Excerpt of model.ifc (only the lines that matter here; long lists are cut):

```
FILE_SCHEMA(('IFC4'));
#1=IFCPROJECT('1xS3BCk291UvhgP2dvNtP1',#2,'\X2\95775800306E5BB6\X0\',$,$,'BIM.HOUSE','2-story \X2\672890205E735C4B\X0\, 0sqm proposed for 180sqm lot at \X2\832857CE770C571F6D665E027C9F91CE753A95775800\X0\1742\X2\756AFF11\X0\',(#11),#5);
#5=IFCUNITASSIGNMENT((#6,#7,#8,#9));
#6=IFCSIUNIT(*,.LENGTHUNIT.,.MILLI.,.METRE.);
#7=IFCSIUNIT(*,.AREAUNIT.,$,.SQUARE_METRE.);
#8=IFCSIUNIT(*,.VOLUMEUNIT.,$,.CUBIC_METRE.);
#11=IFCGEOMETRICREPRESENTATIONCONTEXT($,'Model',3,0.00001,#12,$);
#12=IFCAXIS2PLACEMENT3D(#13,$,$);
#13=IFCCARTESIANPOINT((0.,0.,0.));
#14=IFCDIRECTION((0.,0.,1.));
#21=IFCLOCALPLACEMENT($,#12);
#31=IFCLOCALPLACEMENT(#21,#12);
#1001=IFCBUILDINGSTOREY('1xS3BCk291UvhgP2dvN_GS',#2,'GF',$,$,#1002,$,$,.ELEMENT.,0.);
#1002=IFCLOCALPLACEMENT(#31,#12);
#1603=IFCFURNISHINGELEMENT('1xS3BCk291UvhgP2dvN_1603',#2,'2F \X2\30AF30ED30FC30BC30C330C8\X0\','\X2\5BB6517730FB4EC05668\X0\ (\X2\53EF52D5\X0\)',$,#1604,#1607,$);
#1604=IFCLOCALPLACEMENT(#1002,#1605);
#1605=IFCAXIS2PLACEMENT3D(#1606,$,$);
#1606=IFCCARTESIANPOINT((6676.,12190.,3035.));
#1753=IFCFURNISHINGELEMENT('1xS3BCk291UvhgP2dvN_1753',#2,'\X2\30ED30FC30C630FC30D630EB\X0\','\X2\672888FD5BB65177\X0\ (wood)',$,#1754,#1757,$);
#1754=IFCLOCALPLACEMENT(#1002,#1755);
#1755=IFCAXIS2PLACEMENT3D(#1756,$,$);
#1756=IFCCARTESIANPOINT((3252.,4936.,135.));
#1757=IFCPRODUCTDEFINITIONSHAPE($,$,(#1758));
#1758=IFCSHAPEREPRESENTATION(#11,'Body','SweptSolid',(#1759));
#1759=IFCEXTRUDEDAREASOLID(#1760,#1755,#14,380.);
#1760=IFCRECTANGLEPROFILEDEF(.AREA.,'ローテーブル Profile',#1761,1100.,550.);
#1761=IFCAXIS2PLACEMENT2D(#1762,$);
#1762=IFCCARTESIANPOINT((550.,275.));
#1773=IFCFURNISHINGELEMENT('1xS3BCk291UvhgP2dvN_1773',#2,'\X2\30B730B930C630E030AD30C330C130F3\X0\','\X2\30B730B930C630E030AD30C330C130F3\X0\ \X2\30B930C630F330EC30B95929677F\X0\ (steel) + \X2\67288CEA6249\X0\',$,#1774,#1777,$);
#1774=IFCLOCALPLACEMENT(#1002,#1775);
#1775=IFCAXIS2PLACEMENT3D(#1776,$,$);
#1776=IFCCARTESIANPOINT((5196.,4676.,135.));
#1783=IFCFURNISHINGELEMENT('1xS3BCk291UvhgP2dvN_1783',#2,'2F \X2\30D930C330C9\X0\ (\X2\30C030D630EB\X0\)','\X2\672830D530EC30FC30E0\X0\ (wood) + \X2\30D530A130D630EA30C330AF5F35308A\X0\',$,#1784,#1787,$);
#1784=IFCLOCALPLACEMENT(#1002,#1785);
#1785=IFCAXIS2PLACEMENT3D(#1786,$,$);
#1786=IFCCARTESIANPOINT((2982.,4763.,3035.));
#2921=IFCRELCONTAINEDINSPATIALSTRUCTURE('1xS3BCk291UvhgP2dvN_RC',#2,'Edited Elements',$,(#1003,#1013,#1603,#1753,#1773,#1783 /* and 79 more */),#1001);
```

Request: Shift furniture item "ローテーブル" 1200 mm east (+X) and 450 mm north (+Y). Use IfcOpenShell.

```python
import ifcopenshell
import ifcopenshell.api.geometry
import ifcopenshell.util.placement

model = ifcopenshell.open("model.ifc")

item = model.by_guid("1xS3BCk291UvhgP2dvN_1753")
matrix = ifcopenshell.util.placement.get_local_placement(item.ObjectPlacement)
matrix[0, 3] += 1200.0
matrix[1, 3] += 450.0
ifcopenshell.api.geometry.edit_object_placement(model, product=item, matrix=matrix, is_si=False)

print(ifcopenshell.util.placement.get_local_placement(item.ObjectPlacement).round(3) + 0.0)

model.write("model_edited.ifc")
```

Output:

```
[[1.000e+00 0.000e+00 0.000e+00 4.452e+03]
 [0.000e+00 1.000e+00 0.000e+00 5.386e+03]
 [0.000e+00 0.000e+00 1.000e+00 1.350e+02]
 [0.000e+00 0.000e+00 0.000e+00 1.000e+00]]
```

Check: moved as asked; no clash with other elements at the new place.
